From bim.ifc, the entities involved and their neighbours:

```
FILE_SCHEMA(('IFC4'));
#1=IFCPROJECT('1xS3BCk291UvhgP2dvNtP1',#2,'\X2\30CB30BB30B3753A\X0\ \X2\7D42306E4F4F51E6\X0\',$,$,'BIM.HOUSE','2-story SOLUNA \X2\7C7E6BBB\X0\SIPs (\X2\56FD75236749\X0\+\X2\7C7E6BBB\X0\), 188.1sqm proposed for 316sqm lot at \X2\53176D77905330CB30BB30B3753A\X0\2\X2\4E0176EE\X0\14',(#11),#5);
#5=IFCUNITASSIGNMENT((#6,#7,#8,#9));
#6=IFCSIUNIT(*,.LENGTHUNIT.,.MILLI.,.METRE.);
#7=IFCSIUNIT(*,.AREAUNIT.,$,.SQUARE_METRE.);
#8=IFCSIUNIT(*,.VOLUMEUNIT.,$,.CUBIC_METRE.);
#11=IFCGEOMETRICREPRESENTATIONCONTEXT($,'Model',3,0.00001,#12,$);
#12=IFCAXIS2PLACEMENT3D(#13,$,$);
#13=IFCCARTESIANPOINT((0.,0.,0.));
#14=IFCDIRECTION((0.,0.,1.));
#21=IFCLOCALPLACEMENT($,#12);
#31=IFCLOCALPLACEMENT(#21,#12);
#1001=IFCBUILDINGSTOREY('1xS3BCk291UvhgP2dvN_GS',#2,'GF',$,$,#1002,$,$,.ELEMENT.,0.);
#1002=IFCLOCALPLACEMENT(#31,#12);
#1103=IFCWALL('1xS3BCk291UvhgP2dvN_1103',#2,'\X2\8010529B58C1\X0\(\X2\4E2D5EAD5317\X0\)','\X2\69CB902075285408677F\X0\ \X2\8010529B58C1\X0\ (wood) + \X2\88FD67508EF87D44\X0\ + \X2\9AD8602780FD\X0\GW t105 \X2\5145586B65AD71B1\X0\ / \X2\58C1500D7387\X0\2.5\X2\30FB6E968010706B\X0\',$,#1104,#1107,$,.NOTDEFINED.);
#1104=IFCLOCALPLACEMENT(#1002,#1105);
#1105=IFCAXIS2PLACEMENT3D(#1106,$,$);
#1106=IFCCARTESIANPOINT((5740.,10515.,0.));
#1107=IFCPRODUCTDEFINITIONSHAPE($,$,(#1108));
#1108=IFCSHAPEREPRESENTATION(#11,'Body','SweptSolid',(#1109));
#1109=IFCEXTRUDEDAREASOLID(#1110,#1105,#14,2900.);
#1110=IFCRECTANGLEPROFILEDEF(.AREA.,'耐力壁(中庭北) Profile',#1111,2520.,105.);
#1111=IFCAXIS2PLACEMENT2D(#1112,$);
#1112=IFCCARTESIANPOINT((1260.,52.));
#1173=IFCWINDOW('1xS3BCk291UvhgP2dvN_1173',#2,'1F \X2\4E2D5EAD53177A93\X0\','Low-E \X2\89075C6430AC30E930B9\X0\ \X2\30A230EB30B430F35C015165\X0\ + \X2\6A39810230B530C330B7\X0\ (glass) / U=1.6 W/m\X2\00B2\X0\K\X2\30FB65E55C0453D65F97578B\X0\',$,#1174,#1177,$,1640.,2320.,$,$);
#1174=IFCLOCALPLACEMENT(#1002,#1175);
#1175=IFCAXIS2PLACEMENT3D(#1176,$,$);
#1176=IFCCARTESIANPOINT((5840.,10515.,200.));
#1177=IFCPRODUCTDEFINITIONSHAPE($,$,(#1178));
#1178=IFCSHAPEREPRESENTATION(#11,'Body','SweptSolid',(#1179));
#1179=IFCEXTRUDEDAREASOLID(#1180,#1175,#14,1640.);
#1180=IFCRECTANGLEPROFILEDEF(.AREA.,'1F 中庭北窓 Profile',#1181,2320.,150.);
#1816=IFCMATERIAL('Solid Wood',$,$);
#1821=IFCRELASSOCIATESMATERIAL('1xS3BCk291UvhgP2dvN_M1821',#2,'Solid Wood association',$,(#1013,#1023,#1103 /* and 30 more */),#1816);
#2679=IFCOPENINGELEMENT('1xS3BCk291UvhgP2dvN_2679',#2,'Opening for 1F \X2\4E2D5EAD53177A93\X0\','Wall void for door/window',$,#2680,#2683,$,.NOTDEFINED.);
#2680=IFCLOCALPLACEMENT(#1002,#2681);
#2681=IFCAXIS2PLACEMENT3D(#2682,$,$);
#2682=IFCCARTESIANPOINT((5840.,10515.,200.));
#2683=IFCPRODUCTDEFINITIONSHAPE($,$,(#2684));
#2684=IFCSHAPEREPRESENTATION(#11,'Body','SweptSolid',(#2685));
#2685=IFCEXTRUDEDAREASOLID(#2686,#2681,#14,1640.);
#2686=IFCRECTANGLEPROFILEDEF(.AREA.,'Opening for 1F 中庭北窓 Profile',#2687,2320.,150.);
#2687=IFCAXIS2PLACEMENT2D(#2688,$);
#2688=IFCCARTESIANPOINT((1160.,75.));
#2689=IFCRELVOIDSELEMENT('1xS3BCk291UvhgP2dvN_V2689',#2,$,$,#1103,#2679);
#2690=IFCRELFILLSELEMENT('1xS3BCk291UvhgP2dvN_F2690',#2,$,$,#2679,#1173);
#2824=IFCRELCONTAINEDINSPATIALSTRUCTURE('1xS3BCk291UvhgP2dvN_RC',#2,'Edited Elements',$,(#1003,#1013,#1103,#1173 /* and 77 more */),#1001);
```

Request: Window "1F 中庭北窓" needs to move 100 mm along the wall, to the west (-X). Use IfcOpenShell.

```python
import ifcopenshell
import ifcopenshell.api.geometry
import ifcopenshell.util.placement
import ifcopenshell.util.unit

model = ifcopenshell.open("bim.ifc")
unit_scale = ifcopenshell.util.unit.calculate_unit_scale(model)

window = model.by_id(1173)
opening = window.FillsVoids[0].RelatingOpeningElement
wall = opening.VoidsElements[0].RelatingBuildingElement

wall_matrix = ifcopenshell.util.placement.get_local_placement(wall.ObjectPlacement)
shift = wall_matrix[:3, 0] * -0.1 / unit_scale
before = ifcopenshell.util.placement.get_local_placement(window.ObjectPlacement)[:3, 3].copy()

# The window is not placed relative to its opening, so move both.
for product in (opening, window):
    matrix = ifcopenshell.util.placement.get_local_placement(product.ObjectPlacement)
    matrix[:3, 3] += shift
    ifcopenshell.api.geometry.edit_object_placement(model, product=product, matrix=matrix, is_si=False)

after = ifcopenshell.util.placement.get_local_placement(window.ObjectPlacement)[:3, 3]
print("window moved by", (after - before).round(3) + 0.0)

model.write("bim-out.ifc")
```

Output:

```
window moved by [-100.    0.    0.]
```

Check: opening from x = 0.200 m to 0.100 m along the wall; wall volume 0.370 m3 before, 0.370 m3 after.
